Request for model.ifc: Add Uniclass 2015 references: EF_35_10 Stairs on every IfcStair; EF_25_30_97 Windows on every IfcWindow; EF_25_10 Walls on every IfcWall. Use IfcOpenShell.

First a look at what the model holds.

```python
import ifcopenshell

model = ifcopenshell.open("model.ifc")
print(model.schema)
print("classifications:", [c.Name for c in model.by_type("IfcClassification")])
for ifc_class in ("IfcDoor", "IfcRoof", "IfcStair", "IfcWall", "IfcWindow"):
    print(ifc_class, len(model.by_type(ifc_class)))
```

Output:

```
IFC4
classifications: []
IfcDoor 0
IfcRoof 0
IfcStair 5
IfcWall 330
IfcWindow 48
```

```python
import ifcopenshell
import ifcopenshell.api.classification

model = ifcopenshell.open("model.ifc")

system = ifcopenshell.api.classification.add_classification(model, classification="Uniclass 2015")

codes = {
    "IfcStair": ("EF_35_10", "Stairs"),
    "IfcWindow": ("EF_25_30_97", "Windows"),
    "IfcWall": ("EF_25_10", "Walls"),
}
for ifc_class, (code, name) in codes.items():
    products = model.by_type(ifc_class)
    ifcopenshell.api.classification.add_reference(
        model, products=products, classification=system, identification=code, name=name
    )
    print(code, len(products))

model.write("model_v2.ifc")
```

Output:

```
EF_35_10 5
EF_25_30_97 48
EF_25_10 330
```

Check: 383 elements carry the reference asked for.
